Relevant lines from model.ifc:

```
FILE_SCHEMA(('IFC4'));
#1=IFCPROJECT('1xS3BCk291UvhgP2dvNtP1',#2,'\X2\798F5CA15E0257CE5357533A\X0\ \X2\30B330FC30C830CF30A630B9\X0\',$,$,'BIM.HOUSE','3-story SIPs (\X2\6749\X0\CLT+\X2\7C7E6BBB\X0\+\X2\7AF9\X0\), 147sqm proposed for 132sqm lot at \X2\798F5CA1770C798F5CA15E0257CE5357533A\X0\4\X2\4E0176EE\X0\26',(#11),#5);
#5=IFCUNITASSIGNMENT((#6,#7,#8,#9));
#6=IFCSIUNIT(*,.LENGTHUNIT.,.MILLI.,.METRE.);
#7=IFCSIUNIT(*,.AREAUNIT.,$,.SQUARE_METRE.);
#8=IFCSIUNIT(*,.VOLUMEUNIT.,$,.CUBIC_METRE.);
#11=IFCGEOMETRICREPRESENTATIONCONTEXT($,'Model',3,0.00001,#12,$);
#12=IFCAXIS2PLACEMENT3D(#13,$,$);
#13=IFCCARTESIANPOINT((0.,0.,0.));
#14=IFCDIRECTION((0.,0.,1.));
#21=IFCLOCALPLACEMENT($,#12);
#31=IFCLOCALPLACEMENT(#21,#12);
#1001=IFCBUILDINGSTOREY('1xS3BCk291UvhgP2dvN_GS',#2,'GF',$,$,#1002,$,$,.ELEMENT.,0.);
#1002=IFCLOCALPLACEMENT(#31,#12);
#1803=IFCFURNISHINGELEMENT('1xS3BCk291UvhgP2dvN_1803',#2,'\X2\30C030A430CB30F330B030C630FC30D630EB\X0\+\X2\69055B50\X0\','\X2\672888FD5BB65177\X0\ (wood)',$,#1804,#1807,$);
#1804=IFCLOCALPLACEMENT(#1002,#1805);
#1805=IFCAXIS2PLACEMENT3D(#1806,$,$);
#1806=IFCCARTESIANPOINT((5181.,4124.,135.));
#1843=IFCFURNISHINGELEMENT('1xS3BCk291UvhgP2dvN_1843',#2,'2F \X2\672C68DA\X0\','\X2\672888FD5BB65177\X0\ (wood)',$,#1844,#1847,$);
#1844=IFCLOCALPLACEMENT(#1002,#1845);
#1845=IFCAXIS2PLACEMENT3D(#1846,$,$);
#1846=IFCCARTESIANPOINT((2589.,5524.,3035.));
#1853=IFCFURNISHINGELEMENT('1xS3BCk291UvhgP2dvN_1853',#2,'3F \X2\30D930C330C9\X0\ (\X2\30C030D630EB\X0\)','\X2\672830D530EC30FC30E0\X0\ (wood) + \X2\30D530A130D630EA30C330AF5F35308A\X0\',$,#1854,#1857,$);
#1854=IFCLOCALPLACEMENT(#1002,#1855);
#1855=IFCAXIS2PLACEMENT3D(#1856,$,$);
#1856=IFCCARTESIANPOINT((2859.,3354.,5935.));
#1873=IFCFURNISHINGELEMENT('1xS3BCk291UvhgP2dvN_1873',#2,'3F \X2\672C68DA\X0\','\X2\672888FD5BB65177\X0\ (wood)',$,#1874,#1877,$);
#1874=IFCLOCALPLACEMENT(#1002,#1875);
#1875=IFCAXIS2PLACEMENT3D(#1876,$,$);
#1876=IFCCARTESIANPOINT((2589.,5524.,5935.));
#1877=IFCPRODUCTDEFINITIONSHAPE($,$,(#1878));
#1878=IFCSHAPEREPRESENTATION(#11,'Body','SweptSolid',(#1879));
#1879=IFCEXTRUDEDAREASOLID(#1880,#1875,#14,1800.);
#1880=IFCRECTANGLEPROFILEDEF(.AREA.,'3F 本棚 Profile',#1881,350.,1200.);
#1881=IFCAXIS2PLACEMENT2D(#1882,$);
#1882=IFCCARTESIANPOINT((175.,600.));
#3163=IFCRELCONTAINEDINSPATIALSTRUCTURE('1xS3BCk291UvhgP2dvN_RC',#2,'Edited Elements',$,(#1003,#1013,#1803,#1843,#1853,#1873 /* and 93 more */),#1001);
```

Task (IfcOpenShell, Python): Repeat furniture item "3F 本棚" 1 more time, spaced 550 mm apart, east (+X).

```python
import numpy as np
import ifcopenshell
import ifcopenshell.api.geometry
import ifcopenshell.api.root
import ifcopenshell.util.element
import ifcopenshell.util.placement

model = ifcopenshell.open("model.ifc")


def reuse_history(source, copy):
    """copy_class also copies each property set's owner history, people and application; keep the originals."""
    for rel in copy.IsDefinedBy:
        if rel.is_a("IfcRelDefinesByProperties") and (history := rel.RelatingPropertyDefinition.OwnerHistory):
            rel.RelatingPropertyDefinition.OwnerHistory = source.OwnerHistory
            ifcopenshell.util.element.remove_deep2(model, history)


source = model.by_id(1873)
base = ifcopenshell.util.placement.get_local_placement(source.ObjectPlacement)
step = np.array([1.0, 0.0, 0.0]) * 550.0

for i in range(1, 2):
    copy = ifcopenshell.api.root.copy_class(model, product=source)
    copy.Representation = ifcopenshell.util.element.copy_deep(
        model, source.Representation, exclude=["IfcGeometricRepresentationContext", "IfcRepresentationMap"]
    )
    reuse_history(source, copy)
    matrix = base.copy()
    matrix[:3, 3] += i * step
    print("added at", matrix[:3, 3].round(3) + 0.0)
    ifcopenshell.api.geometry.edit_object_placement(model, product=copy, matrix=matrix, is_si=False)

model.write("model_edited.ifc")
```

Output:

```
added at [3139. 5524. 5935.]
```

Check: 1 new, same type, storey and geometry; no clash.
